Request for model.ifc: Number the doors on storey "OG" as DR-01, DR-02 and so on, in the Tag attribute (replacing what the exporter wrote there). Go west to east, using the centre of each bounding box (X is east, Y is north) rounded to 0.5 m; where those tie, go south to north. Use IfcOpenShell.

First a look at what the model holds.

```python
import ifcopenshell
import ifcopenshell.util.element
import ifcopenshell.util.placement

model = ifcopenshell.open("model.ifc")
print(model.schema)
storey = next(s for s in model.by_type("IfcBuildingStorey") if s.Name == "OG")
doors = [e for e in ifcopenshell.util.element.get_decomposition(storey) if e.is_a("IfcDoor")]
for e in sorted(doors, key=lambda e: e.id()):
    origin = ifcopenshell.util.placement.get_local_placement(e.ObjectPlacement)[:3, 3]
    print(e.id(), e.Tag, e.Name, origin.round(2) + 0.0, sep=" | ")
```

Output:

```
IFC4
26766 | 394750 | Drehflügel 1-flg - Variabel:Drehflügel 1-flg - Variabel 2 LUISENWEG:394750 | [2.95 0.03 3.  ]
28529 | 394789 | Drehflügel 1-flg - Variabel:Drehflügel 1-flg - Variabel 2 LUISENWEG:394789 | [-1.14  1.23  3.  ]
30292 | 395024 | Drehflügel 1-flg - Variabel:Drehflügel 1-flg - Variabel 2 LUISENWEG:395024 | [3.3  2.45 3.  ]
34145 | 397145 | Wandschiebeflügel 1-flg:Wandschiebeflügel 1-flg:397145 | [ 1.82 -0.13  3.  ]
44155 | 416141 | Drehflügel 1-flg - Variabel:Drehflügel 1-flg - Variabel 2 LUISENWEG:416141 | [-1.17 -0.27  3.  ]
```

```python
import ifcopenshell
import ifcopenshell.geom
import ifcopenshell.util.element
import ifcopenshell.util.shape

model = ifcopenshell.open("model.ifc")
settings = ifcopenshell.geom.settings()
settings.set("use-world-coords", True)


def centre(element):
    shape = ifcopenshell.geom.create_shape(settings, element)
    return ifcopenshell.util.shape.get_bbox_centroid(shape.geometry)


storey = next(s for s in model.by_type("IfcBuildingStorey") if s.Name == "OG")
doors = [e for e in ifcopenshell.util.element.get_decomposition(storey) if e.is_a("IfcDoor")]

# Insertion points can sit at a corner or the storey origin, so sort by the geometry (in metres).
centres = {e: centre(e) for e in doors}
doors.sort(key=lambda e: (round(centres[e][0] / 0.5), centres[e][1]))

for i, e in enumerate(doors, start=1):
    number = f"DR-{i:02d}"
    e.Tag = number
    print(e.id(), number)

model.write("model_v2.ifc")
```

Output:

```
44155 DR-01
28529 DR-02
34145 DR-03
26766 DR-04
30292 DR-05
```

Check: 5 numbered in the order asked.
